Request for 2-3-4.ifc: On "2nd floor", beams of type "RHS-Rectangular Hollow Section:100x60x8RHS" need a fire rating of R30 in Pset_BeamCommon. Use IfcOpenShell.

First a look at what the model holds.

```python
import ifcopenshell
import ifcopenshell.util.element

model = ifcopenshell.open("2-3-4.ifc")
print(model.schema)
storey = next(s for s in model.by_type("IfcBuildingStorey") if s.Name == "2nd floor")
beams = [e for e in ifcopenshell.util.element.get_decomposition(storey) if e.is_a("IfcBeam")]
seen = {}
for e in beams:
    element_type = ifcopenshell.util.element.get_type(e)
    key = (element_type.Name if element_type != e and element_type else None, ifcopenshell.util.element.get_pset(e, "Pset_BeamCommon", "FireRating"))
    seen[key] = seen.get(key, 0) + 1
for (name, value), count in sorted(seen.items(), key=str):
    print(count, "x", name, "|", value)
```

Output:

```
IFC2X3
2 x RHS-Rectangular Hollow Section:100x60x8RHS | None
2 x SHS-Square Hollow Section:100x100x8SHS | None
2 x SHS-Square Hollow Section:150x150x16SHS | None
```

```python
import ifcopenshell
import ifcopenshell.api.pset
import ifcopenshell.util.element

model = ifcopenshell.open("2-3-4.ifc")

storey = next(s for s in model.by_type("IfcBuildingStorey") if s.Name == "2nd floor")
beams = [e for e in ifcopenshell.util.element.get_decomposition(storey) if e.is_a("IfcBeam")]

count = 0
for e in beams:
    element_type = ifcopenshell.util.element.get_type(e)
    if element_type in (None, e) or element_type.Name != "RHS-Rectangular Hollow Section:100x60x8RHS":
        continue
    # add_pset returns the element's existing set when there is one.
    pset = ifcopenshell.api.pset.add_pset(model, product=e, name="Pset_BeamCommon")
    ifcopenshell.api.pset.edit_pset(model, pset=pset, properties={"FireRating": "R30"})
    count += 1

print(count, "beams updated")

model.write("2-3-4_edited.ifc")
```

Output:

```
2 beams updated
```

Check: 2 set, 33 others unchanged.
